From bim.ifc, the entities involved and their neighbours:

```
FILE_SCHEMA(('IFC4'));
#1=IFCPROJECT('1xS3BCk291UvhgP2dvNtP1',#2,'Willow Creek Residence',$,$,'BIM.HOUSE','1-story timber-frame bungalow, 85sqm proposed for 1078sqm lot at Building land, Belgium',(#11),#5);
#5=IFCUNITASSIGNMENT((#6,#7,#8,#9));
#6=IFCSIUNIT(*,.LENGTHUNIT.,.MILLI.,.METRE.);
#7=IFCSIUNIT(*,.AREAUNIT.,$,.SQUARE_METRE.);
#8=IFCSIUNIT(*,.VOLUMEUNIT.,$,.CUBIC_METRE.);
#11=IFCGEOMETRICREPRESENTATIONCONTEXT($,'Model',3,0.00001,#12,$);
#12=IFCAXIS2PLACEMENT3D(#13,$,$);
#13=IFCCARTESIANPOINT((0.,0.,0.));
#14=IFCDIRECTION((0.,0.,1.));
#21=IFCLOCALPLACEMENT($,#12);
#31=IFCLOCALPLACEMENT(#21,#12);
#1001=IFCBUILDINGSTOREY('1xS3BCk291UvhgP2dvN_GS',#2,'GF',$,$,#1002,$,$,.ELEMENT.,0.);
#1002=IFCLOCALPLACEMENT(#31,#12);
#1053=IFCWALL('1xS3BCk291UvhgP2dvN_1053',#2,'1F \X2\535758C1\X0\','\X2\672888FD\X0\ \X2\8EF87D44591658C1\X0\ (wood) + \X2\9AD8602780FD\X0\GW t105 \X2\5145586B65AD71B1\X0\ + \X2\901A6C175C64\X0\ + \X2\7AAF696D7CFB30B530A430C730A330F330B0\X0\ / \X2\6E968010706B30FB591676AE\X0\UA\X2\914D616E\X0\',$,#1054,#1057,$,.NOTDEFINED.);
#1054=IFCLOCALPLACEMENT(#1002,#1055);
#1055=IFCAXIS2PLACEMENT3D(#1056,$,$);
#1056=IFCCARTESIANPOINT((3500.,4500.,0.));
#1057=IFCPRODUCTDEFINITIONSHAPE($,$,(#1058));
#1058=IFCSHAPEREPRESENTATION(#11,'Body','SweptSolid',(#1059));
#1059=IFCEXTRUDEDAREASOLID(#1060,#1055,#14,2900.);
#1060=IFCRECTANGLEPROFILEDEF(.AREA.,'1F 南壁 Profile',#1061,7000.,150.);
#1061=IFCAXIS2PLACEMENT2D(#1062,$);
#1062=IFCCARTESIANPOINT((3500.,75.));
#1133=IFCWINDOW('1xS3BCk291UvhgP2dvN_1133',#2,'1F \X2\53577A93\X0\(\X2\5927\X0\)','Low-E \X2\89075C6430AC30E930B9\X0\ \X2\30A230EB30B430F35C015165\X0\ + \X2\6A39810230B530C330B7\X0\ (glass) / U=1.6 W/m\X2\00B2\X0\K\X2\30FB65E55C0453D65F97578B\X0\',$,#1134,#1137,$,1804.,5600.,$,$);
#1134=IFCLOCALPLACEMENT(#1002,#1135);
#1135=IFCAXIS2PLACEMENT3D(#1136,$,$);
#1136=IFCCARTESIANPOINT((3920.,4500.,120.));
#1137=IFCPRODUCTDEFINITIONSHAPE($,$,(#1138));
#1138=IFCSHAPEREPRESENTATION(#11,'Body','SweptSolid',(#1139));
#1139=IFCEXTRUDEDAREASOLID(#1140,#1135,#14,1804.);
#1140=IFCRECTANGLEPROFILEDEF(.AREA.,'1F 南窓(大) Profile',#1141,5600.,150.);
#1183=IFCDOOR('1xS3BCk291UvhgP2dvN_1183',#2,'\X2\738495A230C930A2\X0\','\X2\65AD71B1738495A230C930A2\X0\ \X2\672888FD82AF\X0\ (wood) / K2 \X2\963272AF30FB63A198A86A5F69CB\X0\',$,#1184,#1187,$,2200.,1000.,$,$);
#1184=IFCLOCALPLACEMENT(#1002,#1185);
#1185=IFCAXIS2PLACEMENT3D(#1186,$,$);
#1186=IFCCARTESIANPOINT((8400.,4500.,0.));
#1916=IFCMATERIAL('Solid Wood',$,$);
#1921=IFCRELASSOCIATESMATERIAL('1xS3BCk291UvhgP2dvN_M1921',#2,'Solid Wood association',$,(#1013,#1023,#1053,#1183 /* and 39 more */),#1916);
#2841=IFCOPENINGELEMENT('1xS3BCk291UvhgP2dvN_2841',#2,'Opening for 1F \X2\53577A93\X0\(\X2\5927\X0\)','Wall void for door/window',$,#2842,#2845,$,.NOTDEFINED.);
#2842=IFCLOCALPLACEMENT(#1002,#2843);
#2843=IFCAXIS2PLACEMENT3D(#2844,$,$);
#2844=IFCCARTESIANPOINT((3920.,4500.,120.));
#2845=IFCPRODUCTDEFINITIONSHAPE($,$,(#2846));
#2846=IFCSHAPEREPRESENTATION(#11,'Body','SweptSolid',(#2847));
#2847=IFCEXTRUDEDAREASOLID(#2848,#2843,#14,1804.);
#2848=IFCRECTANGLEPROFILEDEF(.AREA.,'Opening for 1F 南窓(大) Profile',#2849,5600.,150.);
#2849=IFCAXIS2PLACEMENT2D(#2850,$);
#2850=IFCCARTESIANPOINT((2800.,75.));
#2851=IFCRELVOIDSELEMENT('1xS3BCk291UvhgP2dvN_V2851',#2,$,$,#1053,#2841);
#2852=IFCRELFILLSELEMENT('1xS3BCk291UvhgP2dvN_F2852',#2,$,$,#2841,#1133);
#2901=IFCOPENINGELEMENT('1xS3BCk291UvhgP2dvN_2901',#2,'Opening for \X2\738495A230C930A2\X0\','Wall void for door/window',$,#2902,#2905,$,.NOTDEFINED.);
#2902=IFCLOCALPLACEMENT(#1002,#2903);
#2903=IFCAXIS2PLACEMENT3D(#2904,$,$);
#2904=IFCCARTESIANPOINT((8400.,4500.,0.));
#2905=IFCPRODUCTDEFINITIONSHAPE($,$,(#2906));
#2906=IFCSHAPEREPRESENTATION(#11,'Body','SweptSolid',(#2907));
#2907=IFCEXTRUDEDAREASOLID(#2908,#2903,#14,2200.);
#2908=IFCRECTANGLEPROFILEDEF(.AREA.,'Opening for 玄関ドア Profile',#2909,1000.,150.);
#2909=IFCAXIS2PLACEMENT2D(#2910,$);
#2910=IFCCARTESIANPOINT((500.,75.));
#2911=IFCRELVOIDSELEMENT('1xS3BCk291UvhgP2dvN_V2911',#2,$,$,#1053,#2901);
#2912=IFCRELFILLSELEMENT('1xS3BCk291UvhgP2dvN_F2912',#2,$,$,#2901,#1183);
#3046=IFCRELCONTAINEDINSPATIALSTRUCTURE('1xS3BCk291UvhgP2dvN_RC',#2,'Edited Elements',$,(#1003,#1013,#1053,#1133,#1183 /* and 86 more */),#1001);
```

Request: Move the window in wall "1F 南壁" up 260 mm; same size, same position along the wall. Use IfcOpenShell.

```python
import numpy as np
import ifcopenshell
import ifcopenshell.api.geometry
import ifcopenshell.util.placement
import ifcopenshell.util.unit

model = ifcopenshell.open("bim.ifc")
unit_scale = ifcopenshell.util.unit.calculate_unit_scale(model)

window = model.by_guid("1xS3BCk291UvhgP2dvN_1133")
opening = window.FillsVoids[0].RelatingOpeningElement
dz = 0.26 / unit_scale

shift = np.array([0.0, 0.0, dz])
# The window is not placed relative to its opening, so move both.
for product in (opening, window):
    matrix = ifcopenshell.util.placement.get_local_placement(product.ObjectPlacement)
    matrix[:3, 3] += shift
    ifcopenshell.api.geometry.edit_object_placement(model, product=product, matrix=matrix, is_si=False)

print(f"moved by {dz * unit_scale:+.3f} m")

model.write("bim_edited.ifc")
```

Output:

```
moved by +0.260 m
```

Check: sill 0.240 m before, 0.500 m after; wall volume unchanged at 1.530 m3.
